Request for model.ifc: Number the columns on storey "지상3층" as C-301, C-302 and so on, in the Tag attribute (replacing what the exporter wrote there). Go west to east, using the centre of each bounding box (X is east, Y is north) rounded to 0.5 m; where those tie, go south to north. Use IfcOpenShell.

First a look at what the model holds.

```python
import ifcopenshell
import ifcopenshell.util.element
import ifcopenshell.util.placement

model = ifcopenshell.open("model.ifc")
print(model.schema)
storey = next(s for s in model.by_type("IfcBuildingStorey") if s.Name == "지상3층")
columns = [e for e in ifcopenshell.util.element.get_decomposition(storey) if e.is_a("IfcColumn")]
for e in sorted(columns, key=lambda e: e.id()):
    origin = ifcopenshell.util.placement.get_local_placement(e.ObjectPlacement)[:3, 3]
    print(e.id(), e.Tag, e.Name, origin.round(2) + 0.0, sep=" | ")
```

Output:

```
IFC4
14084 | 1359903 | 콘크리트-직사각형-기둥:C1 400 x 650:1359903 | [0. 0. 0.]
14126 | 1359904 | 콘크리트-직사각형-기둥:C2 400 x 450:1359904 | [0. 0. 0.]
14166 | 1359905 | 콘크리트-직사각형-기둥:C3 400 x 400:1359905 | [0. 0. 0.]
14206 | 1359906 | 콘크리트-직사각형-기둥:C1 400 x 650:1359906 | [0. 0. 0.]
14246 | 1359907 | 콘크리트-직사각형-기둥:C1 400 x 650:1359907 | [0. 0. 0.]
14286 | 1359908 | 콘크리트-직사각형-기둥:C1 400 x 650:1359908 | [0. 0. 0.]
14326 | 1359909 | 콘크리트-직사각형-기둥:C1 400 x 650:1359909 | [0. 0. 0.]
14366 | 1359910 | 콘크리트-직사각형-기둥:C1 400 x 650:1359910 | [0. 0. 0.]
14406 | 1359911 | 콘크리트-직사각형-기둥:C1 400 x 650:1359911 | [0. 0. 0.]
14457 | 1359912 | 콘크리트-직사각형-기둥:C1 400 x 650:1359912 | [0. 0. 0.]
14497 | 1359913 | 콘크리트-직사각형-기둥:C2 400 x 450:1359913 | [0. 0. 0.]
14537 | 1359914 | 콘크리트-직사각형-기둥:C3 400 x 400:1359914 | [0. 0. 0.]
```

```python
import ifcopenshell
import ifcopenshell.geom
import ifcopenshell.util.element
import ifcopenshell.util.shape

model = ifcopenshell.open("model.ifc")
settings = ifcopenshell.geom.settings()
settings.set("use-world-coords", True)


def centre(element):
    shape = ifcopenshell.geom.create_shape(settings, element)
    return ifcopenshell.util.shape.get_bbox_centroid(shape.geometry)


storey = next(s for s in model.by_type("IfcBuildingStorey") if s.Name == "지상3층")
columns = [e for e in ifcopenshell.util.element.get_decomposition(storey) if e.is_a("IfcColumn")]

# Insertion points can sit at a corner or the storey origin, so sort by the geometry (in metres).
centres = {e: centre(e) for e in columns}
columns.sort(key=lambda e: (round(centres[e][0] / 0.5), centres[e][1]))

for i, e in enumerate(columns, start=1):
    number = f"C-3{i:02d}"
    e.Tag = number
    print(e.id(), number)

model.write("model-out.ifc")
```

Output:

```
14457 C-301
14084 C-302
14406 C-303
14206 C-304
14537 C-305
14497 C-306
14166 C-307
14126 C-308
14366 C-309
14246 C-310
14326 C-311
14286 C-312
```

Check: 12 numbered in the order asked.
